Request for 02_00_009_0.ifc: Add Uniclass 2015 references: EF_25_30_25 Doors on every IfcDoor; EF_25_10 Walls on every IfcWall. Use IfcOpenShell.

First a look at what the model holds.

```python
import ifcopenshell

model = ifcopenshell.open("02_00_009_0.ifc")
print(model.schema)
print("classifications:", [c.Name for c in model.by_type("IfcClassification")])
for ifc_class in ("IfcDoor", "IfcRoof", "IfcStair", "IfcWall", "IfcWindow"):
    print(ifc_class, len(model.by_type(ifc_class)))
```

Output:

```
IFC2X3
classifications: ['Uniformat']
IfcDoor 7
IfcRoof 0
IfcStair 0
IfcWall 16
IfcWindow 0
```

```python
import ifcopenshell
import ifcopenshell.api.classification

model = ifcopenshell.open("02_00_009_0.ifc")

# IFC2X3 requires Source and Edition and has no link from the project to the system.
system = model.create_entity("IfcClassification", Source="NBS", Edition="2015", Name="Uniclass 2015")

codes = {
    "IfcDoor": ("EF_25_30_25", "Doors"),
    "IfcWall": ("EF_25_10", "Walls"),
}
for ifc_class, (code, name) in codes.items():
    products = model.by_type(ifc_class)
    ifcopenshell.api.classification.add_reference(
        model, products=products, classification=system, identification=code, name=name
    )
    print(code, len(products))

model.write("02_00_009_0_rev.ifc")
```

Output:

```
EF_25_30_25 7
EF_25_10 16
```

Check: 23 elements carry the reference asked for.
